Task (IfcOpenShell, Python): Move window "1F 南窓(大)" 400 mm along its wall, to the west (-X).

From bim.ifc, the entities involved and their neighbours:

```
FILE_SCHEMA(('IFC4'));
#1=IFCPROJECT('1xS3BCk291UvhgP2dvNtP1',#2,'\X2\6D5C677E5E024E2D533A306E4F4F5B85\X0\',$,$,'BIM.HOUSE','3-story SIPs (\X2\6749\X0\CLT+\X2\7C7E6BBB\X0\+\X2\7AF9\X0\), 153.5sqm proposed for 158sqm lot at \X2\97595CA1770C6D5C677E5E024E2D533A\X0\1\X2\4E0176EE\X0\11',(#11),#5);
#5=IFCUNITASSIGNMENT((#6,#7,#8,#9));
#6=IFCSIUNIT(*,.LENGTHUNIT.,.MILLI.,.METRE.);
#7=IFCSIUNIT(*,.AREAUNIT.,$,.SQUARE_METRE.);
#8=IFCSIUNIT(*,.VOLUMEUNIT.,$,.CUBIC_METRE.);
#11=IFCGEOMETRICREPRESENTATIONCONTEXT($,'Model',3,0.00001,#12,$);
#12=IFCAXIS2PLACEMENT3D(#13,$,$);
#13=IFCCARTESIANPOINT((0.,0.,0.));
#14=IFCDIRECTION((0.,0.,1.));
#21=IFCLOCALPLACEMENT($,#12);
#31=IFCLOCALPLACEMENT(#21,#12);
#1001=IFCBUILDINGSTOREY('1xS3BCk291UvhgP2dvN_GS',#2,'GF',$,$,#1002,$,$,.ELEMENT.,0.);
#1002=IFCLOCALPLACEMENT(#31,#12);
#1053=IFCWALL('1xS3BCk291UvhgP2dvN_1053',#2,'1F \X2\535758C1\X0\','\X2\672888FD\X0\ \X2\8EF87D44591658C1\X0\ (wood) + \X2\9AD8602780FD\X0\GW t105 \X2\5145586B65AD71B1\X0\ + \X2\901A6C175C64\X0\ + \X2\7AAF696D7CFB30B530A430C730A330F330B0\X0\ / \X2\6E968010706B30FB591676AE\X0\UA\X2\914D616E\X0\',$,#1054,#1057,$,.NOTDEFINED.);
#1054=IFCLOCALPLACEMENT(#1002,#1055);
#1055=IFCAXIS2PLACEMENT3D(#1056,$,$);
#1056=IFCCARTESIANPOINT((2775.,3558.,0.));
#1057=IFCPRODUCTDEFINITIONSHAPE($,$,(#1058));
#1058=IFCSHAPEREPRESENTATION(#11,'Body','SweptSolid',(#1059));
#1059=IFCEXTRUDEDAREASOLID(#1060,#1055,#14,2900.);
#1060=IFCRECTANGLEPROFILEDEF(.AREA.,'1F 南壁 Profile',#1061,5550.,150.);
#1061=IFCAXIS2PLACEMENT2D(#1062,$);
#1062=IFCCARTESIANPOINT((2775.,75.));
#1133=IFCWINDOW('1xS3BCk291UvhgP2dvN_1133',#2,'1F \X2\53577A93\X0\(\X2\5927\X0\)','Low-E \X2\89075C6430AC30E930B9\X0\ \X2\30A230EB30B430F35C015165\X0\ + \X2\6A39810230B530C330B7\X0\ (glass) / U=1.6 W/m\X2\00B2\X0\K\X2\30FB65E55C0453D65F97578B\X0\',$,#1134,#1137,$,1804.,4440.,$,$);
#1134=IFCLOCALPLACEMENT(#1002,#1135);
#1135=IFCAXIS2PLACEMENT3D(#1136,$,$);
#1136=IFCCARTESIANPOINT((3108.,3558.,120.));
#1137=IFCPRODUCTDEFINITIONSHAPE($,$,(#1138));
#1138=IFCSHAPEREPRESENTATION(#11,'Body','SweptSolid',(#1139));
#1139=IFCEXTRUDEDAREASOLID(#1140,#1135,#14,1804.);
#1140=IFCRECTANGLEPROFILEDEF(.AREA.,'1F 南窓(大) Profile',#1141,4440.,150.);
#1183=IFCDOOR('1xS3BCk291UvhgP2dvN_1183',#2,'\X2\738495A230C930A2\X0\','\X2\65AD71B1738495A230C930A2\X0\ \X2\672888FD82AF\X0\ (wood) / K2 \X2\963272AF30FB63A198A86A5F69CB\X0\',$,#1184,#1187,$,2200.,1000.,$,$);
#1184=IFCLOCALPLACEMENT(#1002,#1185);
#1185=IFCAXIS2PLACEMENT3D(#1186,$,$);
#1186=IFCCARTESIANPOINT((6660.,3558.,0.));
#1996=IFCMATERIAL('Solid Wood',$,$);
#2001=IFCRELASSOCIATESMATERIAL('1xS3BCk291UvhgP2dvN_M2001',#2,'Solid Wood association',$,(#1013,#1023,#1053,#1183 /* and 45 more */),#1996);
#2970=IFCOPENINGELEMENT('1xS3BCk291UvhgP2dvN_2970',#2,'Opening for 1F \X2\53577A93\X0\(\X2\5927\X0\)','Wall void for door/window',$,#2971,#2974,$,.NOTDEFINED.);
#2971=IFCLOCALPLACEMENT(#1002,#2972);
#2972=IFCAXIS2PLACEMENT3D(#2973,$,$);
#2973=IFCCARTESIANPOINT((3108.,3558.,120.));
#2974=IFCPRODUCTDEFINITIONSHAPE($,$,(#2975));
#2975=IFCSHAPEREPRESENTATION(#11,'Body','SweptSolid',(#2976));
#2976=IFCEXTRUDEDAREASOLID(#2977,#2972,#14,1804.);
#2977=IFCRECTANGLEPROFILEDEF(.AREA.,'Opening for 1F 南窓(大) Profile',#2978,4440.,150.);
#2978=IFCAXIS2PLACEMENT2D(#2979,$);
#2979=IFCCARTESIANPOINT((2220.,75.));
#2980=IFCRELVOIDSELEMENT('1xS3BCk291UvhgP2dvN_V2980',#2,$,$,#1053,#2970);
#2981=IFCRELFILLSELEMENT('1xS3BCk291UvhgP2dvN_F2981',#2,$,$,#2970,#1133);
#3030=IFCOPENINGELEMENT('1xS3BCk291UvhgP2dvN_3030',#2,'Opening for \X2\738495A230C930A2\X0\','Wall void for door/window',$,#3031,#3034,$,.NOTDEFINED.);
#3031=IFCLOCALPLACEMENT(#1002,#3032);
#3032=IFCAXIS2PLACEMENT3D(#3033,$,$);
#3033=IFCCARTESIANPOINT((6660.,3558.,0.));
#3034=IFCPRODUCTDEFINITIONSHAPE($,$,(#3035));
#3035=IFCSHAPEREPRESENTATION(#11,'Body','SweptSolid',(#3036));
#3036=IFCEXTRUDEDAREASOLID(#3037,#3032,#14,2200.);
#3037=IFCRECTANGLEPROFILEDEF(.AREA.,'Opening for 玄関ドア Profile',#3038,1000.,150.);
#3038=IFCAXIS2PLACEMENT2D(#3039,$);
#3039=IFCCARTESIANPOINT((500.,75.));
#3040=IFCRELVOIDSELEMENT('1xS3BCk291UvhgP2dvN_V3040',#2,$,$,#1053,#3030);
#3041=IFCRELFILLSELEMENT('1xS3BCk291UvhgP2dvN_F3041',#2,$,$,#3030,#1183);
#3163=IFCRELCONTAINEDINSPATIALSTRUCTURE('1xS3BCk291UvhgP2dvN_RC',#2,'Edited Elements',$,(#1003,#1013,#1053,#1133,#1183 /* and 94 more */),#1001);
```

```python
import ifcopenshell
import ifcopenshell.api.geometry
import ifcopenshell.util.placement

model = ifcopenshell.open("bim.ifc")

window = model.by_guid("1xS3BCk291UvhgP2dvN_1133")
opening = window.FillsVoids[0].RelatingOpeningElement
wall = opening.VoidsElements[0].RelatingBuildingElement

wall_matrix = ifcopenshell.util.placement.get_local_placement(wall.ObjectPlacement)
shift = wall_matrix[:3, 0] * -400.0
before = ifcopenshell.util.placement.get_local_placement(window.ObjectPlacement)[:3, 3].copy()

# The window is not placed relative to its opening, so move both.
for product in (opening, window):
    matrix = ifcopenshell.util.placement.get_local_placement(product.ObjectPlacement)
    matrix[:3, 3] += shift
    ifcopenshell.api.geometry.edit_object_placement(model, product=product, matrix=matrix, is_si=False)

after = ifcopenshell.util.placement.get_local_placement(window.ObjectPlacement)[:3, 3]
print("window moved by", (after - before).round(3) + 0.0)

model.write("bim_edited.ifc")
```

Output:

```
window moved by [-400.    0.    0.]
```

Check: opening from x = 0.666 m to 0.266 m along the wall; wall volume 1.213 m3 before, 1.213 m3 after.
